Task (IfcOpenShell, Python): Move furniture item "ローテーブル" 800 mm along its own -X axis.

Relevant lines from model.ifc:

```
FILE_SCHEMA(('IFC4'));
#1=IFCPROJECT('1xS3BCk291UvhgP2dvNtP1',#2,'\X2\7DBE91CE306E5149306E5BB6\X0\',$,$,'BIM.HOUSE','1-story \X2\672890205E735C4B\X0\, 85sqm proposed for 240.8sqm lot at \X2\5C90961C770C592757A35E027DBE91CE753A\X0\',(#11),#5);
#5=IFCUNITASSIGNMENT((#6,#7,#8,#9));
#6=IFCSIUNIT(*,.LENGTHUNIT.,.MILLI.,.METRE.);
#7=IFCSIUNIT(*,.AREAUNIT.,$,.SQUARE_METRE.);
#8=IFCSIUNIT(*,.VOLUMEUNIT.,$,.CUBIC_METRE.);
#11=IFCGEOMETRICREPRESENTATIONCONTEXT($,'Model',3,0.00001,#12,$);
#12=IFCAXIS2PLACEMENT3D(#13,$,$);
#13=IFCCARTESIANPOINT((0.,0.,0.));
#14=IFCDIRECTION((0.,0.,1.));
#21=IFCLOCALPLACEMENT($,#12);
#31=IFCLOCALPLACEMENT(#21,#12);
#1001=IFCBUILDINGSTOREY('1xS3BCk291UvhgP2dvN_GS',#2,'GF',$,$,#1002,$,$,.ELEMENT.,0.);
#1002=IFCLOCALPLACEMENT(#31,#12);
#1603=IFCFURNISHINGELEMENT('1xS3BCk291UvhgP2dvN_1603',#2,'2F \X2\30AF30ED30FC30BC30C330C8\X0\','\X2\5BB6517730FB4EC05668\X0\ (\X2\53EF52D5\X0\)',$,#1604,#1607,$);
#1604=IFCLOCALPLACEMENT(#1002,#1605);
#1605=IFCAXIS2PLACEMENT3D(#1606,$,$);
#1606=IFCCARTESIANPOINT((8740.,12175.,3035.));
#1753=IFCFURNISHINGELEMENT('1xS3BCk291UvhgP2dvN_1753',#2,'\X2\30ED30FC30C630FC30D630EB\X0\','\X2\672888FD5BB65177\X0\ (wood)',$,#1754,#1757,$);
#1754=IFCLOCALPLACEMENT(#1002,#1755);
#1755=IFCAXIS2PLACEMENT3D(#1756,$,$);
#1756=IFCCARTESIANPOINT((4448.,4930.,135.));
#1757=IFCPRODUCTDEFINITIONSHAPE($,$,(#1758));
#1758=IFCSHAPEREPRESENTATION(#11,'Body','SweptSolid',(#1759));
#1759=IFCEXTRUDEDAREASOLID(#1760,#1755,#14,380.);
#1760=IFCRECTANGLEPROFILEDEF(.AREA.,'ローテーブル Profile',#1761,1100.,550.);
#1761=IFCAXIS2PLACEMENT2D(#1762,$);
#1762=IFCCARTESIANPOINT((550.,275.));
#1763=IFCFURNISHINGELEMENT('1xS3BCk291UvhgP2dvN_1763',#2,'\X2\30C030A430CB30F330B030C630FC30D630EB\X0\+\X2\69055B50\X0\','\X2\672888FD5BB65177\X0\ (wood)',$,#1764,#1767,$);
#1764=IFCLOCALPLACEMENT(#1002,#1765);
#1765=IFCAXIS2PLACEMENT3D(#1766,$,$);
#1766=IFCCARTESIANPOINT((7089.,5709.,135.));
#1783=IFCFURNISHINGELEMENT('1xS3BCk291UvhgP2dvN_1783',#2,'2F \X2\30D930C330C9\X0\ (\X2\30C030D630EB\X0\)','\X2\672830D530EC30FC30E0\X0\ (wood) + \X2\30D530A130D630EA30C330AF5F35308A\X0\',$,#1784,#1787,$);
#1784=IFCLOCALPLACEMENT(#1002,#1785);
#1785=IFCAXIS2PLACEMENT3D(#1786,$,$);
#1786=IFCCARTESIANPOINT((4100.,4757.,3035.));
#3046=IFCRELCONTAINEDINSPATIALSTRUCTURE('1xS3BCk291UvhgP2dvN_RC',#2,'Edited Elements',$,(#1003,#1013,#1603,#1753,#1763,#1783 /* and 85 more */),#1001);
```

```python
import ifcopenshell
import ifcopenshell.api.geometry
import ifcopenshell.util.placement

model = ifcopenshell.open("model.ifc")

item = model.by_id(1753)
matrix = ifcopenshell.util.placement.get_local_placement(item.ObjectPlacement)
matrix[:3, 3] -= matrix[:3, 0] * 800.0
ifcopenshell.api.geometry.edit_object_placement(model, product=item, matrix=matrix, is_si=False)

print(ifcopenshell.util.placement.get_local_placement(item.ObjectPlacement).round(3) + 0.0)

model.write("model_rev.ifc")
```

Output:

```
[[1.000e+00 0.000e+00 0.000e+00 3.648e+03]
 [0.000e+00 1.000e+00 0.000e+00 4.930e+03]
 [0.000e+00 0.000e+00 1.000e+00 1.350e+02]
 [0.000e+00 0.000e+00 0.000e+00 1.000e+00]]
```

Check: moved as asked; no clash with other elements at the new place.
